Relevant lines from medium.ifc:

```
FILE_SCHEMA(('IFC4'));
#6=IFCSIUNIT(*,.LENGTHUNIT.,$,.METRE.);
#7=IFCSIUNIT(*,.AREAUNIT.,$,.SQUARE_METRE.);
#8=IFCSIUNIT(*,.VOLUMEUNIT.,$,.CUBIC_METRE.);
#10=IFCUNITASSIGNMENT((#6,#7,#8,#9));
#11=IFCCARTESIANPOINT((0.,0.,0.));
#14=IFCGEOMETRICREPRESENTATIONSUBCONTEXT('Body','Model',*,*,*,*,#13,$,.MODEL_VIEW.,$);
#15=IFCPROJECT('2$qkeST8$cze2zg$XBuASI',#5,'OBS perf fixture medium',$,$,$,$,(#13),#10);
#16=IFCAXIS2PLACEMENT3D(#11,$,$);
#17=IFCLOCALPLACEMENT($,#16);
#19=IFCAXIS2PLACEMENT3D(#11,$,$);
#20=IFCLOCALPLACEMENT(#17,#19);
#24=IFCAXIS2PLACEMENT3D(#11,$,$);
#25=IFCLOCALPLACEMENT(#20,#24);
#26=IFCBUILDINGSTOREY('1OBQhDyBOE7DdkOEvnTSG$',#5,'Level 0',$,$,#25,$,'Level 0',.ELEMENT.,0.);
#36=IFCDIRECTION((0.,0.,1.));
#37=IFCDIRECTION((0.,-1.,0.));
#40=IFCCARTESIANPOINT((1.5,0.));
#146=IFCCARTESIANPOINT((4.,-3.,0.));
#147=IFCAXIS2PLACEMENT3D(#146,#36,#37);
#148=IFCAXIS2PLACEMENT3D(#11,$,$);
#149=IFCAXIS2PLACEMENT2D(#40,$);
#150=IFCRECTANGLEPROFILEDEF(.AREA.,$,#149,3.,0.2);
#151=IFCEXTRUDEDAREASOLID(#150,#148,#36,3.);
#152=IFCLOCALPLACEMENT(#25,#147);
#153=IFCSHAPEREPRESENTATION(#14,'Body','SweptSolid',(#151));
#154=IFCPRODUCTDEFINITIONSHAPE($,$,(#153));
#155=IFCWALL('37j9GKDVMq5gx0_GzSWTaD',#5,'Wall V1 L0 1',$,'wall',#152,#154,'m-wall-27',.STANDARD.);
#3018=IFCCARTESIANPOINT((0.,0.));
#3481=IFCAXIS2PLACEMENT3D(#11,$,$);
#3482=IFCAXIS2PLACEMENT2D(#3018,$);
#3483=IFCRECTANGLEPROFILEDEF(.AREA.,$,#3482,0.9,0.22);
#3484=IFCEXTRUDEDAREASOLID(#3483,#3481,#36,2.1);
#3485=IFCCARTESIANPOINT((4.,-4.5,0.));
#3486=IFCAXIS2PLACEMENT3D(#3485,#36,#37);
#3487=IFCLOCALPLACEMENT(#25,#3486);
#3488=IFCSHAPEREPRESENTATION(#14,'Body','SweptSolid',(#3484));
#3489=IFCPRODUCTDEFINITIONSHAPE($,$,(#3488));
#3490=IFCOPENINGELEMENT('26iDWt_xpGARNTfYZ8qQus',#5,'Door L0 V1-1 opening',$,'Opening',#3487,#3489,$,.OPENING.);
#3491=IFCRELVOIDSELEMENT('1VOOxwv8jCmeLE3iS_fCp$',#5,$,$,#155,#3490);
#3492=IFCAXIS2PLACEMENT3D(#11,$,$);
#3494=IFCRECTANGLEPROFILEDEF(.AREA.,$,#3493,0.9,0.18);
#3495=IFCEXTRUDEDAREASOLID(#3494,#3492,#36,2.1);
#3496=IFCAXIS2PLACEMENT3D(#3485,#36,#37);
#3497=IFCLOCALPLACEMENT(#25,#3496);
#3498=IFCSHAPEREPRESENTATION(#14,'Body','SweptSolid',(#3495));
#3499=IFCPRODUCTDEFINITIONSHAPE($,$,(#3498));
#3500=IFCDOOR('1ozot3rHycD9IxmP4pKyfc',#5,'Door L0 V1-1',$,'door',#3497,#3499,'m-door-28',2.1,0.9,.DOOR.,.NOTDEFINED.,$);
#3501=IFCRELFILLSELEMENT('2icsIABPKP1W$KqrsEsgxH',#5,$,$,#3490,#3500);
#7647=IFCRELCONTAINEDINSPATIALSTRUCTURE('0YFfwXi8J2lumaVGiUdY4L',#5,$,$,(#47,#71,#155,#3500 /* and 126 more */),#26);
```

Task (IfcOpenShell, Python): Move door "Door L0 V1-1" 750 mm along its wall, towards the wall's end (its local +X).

```python
import ifcopenshell
import ifcopenshell.api.geometry
import ifcopenshell.util.placement
import ifcopenshell.util.unit

model = ifcopenshell.open("medium.ifc")
unit_scale = ifcopenshell.util.unit.calculate_unit_scale(model)

door = model.by_guid("1ozot3rHycD9IxmP4pKyfc")
opening = door.FillsVoids[0].RelatingOpeningElement
wall = opening.VoidsElements[0].RelatingBuildingElement

wall_matrix = ifcopenshell.util.placement.get_local_placement(wall.ObjectPlacement)
shift = wall_matrix[:3, 0] * 0.75 / unit_scale
before = ifcopenshell.util.placement.get_local_placement(door.ObjectPlacement)[:3, 3].copy()

# The door is not placed relative to its opening, so move both.
for product in (opening, door):
    matrix = ifcopenshell.util.placement.get_local_placement(product.ObjectPlacement)
    matrix[:3, 3] += shift
    ifcopenshell.api.geometry.edit_object_placement(model, product=product, matrix=matrix, is_si=False)

after = ifcopenshell.util.placement.get_local_placement(door.ObjectPlacement)[:3, 3]
print("door moved by", (after - before).round(3) + 0.0)

model.write("medium_edited.ifc")
```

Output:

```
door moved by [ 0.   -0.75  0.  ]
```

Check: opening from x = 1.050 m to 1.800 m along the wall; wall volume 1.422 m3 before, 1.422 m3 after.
